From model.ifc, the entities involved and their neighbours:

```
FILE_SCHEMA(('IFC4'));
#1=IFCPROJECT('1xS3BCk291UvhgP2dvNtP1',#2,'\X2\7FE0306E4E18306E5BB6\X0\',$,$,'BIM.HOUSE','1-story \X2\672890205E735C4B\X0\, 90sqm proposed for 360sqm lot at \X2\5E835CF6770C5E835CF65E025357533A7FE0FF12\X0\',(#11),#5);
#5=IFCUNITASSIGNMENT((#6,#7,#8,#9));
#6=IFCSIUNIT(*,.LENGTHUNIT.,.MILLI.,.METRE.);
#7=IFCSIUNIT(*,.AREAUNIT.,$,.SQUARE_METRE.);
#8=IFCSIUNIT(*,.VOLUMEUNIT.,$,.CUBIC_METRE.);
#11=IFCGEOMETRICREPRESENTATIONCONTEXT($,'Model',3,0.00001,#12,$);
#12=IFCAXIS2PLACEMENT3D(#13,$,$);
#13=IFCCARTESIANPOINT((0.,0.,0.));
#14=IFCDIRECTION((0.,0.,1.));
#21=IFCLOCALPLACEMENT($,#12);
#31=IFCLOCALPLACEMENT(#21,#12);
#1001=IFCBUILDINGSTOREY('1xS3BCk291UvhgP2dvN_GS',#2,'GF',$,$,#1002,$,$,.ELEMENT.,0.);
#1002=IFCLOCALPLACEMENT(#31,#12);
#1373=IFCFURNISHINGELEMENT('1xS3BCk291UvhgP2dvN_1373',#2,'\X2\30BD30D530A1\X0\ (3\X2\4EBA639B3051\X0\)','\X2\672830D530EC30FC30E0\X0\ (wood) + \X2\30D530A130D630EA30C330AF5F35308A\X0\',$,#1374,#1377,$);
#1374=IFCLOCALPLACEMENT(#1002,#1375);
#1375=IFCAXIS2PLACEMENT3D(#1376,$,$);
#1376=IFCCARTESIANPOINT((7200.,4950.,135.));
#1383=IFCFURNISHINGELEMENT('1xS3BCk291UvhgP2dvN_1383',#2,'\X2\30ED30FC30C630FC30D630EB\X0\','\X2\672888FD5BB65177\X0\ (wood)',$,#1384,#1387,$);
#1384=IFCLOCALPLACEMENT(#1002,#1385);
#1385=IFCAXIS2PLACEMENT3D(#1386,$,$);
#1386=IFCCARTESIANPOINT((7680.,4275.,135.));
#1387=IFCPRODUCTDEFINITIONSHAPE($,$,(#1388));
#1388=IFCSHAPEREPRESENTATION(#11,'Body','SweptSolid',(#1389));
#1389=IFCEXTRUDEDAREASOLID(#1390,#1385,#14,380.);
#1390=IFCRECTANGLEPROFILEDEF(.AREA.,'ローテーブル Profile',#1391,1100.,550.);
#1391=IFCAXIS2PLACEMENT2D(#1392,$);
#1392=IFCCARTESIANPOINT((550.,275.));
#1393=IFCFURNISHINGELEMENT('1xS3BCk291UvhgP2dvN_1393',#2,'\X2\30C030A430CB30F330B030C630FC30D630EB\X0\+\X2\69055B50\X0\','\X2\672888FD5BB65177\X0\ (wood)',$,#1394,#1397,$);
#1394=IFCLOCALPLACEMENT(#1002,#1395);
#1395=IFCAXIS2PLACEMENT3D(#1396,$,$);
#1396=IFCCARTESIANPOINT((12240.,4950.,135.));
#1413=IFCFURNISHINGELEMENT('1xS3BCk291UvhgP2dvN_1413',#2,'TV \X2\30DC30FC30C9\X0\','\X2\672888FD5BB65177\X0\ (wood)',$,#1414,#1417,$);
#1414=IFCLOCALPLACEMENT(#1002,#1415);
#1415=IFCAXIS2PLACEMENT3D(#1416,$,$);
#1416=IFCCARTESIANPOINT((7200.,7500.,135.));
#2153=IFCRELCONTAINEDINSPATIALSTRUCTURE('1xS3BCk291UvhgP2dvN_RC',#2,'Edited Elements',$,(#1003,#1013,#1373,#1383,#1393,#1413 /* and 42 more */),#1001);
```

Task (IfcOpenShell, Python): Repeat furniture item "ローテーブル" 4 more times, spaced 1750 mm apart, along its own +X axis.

```python
import ifcopenshell
import ifcopenshell.api.geometry
import ifcopenshell.api.root
import ifcopenshell.util.element
import ifcopenshell.util.placement

model = ifcopenshell.open("model.ifc")


def reuse_history(source, copy):
    """copy_class also copies each property set's owner history, people and application; keep the originals."""
    for rel in copy.IsDefinedBy:
        if rel.is_a("IfcRelDefinesByProperties") and (history := rel.RelatingPropertyDefinition.OwnerHistory):
            rel.RelatingPropertyDefinition.OwnerHistory = source.OwnerHistory
            ifcopenshell.util.element.remove_deep2(model, history)


source = model.by_guid("1xS3BCk291UvhgP2dvN_1383")
base = ifcopenshell.util.placement.get_local_placement(source.ObjectPlacement)
step = base[:3, 0] * 1750.0

for i in range(1, 5):
    copy = ifcopenshell.api.root.copy_class(model, product=source)
    copy.Representation = ifcopenshell.util.element.copy_deep(
        model, source.Representation, exclude=["IfcGeometricRepresentationContext", "IfcRepresentationMap"]
    )
    reuse_history(source, copy)
    matrix = base.copy()
    matrix[:3, 3] += i * step
    print("added at", matrix[:3, 3].round(3) + 0.0)
    ifcopenshell.api.geometry.edit_object_placement(model, product=copy, matrix=matrix, is_si=False)

model.write("model_edited.ifc")
```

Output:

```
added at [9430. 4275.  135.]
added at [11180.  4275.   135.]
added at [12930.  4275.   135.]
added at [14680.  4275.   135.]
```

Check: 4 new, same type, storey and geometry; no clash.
